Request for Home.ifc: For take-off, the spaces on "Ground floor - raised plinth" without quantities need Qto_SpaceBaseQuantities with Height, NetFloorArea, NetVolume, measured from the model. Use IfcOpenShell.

First a look at what the model holds.

```python
import ifcopenshell
import ifcopenshell.util.element
import ifcopenshell.util.unit

model = ifcopenshell.open("Home.ifc")
print(model.schema)
for unit_type in ("LENGTHUNIT", "AREAUNIT", "VOLUMEUNIT"):
    print(unit_type, ifcopenshell.util.unit.calculate_unit_scale(model, unit_type))
storey = next(s for s in model.by_type("IfcBuildingStorey") if s.Name == "Ground floor - raised plinth")
spaces = [e for e in ifcopenshell.util.element.get_decomposition(storey) if e.is_a("IfcSpace")]
for e in sorted(spaces, key=lambda e: e.id()):
    print(e.id(), e.is_a(), e.Name, list(ifcopenshell.util.element.get_psets(e, qtos_only=True)), sep=" | ")
```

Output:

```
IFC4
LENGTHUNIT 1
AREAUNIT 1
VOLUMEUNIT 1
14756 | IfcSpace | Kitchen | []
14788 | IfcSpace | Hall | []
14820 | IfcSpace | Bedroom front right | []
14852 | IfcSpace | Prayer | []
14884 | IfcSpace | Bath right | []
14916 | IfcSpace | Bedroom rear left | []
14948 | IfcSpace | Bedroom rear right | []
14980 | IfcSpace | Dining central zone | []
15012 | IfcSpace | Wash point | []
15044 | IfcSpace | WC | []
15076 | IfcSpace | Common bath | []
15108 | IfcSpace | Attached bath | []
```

```python
import ifcopenshell
import ifcopenshell.api.pset
import ifcopenshell.geom
import ifcopenshell.util.element
import ifcopenshell.util.shape
import ifcopenshell.util.unit

model = ifcopenshell.open("Home.ifc")
unit_scale = ifcopenshell.util.unit.calculate_unit_scale(model)
area_scale = ifcopenshell.util.unit.calculate_unit_scale(model, "AREAUNIT")
volume_scale = ifcopenshell.util.unit.calculate_unit_scale(model, "VOLUMEUNIT")
settings = ifcopenshell.geom.settings()

storey = next(s for s in model.by_type("IfcBuildingStorey") if s.Name == "Ground floor - raised plinth")
spaces = [e for e in ifcopenshell.util.element.get_decomposition(storey) if e.is_a("IfcSpace")]

for e in sorted(spaces, key=lambda e: e.id()):
    if ifcopenshell.util.element.get_psets(e, qtos_only=True, should_inherit=False):
        continue
    # Geometry comes back in metres, in the element's own axes.
    shape = ifcopenshell.geom.create_shape(settings, e)
    values = {
        "Height": ifcopenshell.util.shape.get_z(shape.geometry) / unit_scale,
        "NetFloorArea": ifcopenshell.util.shape.get_footprint_area(shape.geometry) / area_scale,
        "NetVolume": ifcopenshell.util.shape.get_volume(shape.geometry) / volume_scale,
    }
    qto = ifcopenshell.api.pset.add_qto(model, product=e, name="Qto_SpaceBaseQuantities")
    ifcopenshell.api.pset.edit_qto(model, qto=qto, properties=values)
    print(e.id(), {k: round(v, 3) for k, v in values.items()})

model.write("Home-out.ifc")
```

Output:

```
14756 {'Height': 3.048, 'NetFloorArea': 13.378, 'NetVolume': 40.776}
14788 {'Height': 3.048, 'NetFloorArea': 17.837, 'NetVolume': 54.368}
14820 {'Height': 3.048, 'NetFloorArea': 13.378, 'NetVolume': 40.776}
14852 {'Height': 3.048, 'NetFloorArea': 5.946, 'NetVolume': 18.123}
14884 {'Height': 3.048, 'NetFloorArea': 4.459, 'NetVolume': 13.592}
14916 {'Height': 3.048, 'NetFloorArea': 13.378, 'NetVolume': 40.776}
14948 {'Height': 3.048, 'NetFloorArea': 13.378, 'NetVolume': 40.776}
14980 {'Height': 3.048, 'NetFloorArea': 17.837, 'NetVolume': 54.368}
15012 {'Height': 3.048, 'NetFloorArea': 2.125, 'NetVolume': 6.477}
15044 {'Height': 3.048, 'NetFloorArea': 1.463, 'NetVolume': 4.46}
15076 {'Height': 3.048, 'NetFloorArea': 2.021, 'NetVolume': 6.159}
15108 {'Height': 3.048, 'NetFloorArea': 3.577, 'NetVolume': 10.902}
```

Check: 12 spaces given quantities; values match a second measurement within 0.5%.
